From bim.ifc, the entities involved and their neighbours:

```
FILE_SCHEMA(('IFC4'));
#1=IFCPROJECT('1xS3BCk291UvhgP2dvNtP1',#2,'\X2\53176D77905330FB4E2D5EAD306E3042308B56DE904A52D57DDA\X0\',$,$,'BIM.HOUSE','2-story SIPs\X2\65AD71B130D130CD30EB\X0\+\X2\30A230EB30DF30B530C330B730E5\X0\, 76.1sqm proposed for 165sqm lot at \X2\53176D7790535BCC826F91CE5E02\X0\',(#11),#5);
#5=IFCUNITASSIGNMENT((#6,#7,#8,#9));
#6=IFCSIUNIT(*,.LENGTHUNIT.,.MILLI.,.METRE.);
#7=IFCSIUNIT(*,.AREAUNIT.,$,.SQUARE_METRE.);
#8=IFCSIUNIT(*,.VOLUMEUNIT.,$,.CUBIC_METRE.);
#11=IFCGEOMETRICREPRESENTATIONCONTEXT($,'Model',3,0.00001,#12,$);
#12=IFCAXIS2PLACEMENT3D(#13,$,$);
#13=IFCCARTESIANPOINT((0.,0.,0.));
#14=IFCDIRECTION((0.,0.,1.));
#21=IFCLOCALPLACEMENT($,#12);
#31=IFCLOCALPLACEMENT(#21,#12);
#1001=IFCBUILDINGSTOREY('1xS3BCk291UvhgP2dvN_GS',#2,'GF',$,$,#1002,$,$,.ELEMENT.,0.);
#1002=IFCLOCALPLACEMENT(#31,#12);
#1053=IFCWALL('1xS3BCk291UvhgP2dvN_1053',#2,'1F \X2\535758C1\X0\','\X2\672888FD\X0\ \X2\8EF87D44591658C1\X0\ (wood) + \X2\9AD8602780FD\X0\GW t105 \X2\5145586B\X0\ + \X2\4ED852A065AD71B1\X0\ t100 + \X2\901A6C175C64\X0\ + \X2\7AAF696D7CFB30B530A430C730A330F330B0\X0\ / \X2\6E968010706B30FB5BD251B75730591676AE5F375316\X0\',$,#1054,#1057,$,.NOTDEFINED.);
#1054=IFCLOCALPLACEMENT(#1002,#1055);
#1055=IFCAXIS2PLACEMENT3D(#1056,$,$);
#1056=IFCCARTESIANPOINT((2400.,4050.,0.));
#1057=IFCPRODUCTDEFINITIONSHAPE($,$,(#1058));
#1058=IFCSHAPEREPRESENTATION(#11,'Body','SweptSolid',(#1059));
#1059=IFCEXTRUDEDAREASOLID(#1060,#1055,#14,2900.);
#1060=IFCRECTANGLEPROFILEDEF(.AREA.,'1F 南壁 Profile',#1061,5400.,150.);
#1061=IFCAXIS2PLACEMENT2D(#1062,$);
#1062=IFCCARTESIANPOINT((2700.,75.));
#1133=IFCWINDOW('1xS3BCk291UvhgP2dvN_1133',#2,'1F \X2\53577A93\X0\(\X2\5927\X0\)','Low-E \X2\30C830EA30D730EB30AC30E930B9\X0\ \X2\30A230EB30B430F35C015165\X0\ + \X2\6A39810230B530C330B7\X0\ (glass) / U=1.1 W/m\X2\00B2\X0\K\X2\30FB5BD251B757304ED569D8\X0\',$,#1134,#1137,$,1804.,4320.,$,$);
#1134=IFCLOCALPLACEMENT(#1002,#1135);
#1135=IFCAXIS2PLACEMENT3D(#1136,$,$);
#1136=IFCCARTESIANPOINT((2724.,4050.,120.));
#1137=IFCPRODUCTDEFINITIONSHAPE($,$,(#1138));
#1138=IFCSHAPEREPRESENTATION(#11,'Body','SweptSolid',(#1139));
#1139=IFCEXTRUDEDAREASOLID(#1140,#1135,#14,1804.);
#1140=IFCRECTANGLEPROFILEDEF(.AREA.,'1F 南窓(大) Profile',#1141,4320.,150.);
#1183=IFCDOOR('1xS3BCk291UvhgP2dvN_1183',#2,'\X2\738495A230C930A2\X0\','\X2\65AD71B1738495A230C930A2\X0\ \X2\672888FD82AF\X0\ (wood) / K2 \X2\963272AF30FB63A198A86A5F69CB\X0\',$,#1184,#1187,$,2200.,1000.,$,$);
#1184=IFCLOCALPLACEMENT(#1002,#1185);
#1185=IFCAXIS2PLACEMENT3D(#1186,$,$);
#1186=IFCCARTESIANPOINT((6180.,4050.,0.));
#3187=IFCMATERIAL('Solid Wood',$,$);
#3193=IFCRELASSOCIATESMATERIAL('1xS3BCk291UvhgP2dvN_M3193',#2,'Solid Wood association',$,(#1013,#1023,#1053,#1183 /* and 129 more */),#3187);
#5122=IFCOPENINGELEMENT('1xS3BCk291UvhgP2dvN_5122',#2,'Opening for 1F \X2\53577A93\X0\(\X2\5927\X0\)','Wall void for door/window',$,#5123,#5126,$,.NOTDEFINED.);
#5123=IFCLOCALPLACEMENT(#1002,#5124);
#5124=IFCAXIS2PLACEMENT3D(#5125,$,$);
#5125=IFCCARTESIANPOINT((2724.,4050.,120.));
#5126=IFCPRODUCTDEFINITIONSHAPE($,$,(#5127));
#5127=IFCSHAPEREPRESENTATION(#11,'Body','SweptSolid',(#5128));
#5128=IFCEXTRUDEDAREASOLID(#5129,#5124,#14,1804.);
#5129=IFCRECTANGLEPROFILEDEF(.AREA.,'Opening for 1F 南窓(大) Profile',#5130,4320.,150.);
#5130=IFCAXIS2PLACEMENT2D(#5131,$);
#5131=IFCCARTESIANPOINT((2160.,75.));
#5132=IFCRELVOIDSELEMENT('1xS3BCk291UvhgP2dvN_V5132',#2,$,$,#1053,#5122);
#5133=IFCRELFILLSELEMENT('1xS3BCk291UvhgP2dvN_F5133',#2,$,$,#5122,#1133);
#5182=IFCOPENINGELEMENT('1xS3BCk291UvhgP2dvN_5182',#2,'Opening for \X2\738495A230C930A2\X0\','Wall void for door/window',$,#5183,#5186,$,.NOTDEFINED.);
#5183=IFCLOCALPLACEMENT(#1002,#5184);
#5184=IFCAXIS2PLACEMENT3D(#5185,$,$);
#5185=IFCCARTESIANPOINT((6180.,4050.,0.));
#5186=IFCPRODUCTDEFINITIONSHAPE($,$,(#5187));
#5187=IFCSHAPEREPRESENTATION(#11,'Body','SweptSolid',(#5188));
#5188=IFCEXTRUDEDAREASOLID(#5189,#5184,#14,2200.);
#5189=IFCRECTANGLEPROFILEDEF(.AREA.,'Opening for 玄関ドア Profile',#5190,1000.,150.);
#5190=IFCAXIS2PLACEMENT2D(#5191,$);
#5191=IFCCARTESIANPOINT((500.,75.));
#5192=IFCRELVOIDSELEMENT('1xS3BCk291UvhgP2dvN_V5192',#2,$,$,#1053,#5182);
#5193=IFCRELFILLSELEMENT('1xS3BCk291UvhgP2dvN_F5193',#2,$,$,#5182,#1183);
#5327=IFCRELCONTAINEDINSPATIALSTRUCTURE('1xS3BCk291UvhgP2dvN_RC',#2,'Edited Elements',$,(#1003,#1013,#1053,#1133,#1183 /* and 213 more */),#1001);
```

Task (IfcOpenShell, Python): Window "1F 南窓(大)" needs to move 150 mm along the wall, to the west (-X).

```python
import ifcopenshell
import ifcopenshell.api.geometry
import ifcopenshell.util.placement

model = ifcopenshell.open("bim.ifc")

window = model.by_guid("1xS3BCk291UvhgP2dvN_1133")
opening = window.FillsVoids[0].RelatingOpeningElement
wall = opening.VoidsElements[0].RelatingBuildingElement

wall_matrix = ifcopenshell.util.placement.get_local_placement(wall.ObjectPlacement)
shift = wall_matrix[:3, 0] * -150.0
before = ifcopenshell.util.placement.get_local_placement(window.ObjectPlacement)[:3, 3].copy()

# The window is not placed relative to its opening, so move both.
for product in (opening, window):
    matrix = ifcopenshell.util.placement.get_local_placement(product.ObjectPlacement)
    matrix[:3, 3] += shift
    ifcopenshell.api.geometry.edit_object_placement(model, product=product, matrix=matrix, is_si=False)

after = ifcopenshell.util.placement.get_local_placement(window.ObjectPlacement)[:3, 3]
print("window moved by", (after - before).round(3) + 0.0)

model.write("bim_updated.ifc")
```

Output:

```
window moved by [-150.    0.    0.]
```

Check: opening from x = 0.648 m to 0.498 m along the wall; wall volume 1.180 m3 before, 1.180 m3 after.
